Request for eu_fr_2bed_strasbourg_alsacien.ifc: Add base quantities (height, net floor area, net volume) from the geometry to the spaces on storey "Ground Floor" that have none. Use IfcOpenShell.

First a look at what the model holds.

```python
import ifcopenshell
import ifcopenshell.util.element
import ifcopenshell.util.unit

model = ifcopenshell.open("eu_fr_2bed_strasbourg_alsacien.ifc")
print(model.schema)
for unit_type in ("LENGTHUNIT", "AREAUNIT", "VOLUMEUNIT"):
    print(unit_type, ifcopenshell.util.unit.calculate_unit_scale(model, unit_type))
storey = next(s for s in model.by_type("IfcBuildingStorey") if s.Name == "Ground Floor")
spaces = [e for e in ifcopenshell.util.element.get_decomposition(storey) if e.is_a("IfcSpace")]
for e in sorted(spaces, key=lambda e: e.id()):
    print(e.id(), e.is_a(), e.Name, list(ifcopenshell.util.element.get_psets(e, qtos_only=True)), sep=" | ")
```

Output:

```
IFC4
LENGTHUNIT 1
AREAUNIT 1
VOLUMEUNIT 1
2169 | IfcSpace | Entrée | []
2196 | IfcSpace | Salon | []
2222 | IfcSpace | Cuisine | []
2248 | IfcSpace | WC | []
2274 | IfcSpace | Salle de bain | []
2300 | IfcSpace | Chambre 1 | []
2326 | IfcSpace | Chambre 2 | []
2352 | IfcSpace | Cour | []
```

```python
import ifcopenshell
import ifcopenshell.api.pset
import ifcopenshell.geom
import ifcopenshell.util.element
import ifcopenshell.util.shape
import ifcopenshell.util.unit

model = ifcopenshell.open("eu_fr_2bed_strasbourg_alsacien.ifc")
unit_scale = ifcopenshell.util.unit.calculate_unit_scale(model)
area_scale = ifcopenshell.util.unit.calculate_unit_scale(model, "AREAUNIT")
volume_scale = ifcopenshell.util.unit.calculate_unit_scale(model, "VOLUMEUNIT")
settings = ifcopenshell.geom.settings()

storey = next(s for s in model.by_type("IfcBuildingStorey") if s.Name == "Ground Floor")
spaces = [e for e in ifcopenshell.util.element.get_decomposition(storey) if e.is_a("IfcSpace")]

for e in sorted(spaces, key=lambda e: e.id()):
    if ifcopenshell.util.element.get_psets(e, qtos_only=True, should_inherit=False):
        continue
    # Geometry comes back in metres, in the element's own axes.
    shape = ifcopenshell.geom.create_shape(settings, e)
    values = {
        "Height": ifcopenshell.util.shape.get_z(shape.geometry) / unit_scale,
        "NetFloorArea": ifcopenshell.util.shape.get_footprint_area(shape.geometry) / area_scale,
        "NetVolume": ifcopenshell.util.shape.get_volume(shape.geometry) / volume_scale,
    }
    qto = ifcopenshell.api.pset.add_qto(model, product=e, name="Qto_SpaceBaseQuantities")
    ifcopenshell.api.pset.edit_qto(model, qto=qto, properties=values)
    print(e.id(), {k: round(v, 3) for k, v in values.items()})

model.write("eu_fr_2bed_strasbourg_alsacien_rev.ifc")
```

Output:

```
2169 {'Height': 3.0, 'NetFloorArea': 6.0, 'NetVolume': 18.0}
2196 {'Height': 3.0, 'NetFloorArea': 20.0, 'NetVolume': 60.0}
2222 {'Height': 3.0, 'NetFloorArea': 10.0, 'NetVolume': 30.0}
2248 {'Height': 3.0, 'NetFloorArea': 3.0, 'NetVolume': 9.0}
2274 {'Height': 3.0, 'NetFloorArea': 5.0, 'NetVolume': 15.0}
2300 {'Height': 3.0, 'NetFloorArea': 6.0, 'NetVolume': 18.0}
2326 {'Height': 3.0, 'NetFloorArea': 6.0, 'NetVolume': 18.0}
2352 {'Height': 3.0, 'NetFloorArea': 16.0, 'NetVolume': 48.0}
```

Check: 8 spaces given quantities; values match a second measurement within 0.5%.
